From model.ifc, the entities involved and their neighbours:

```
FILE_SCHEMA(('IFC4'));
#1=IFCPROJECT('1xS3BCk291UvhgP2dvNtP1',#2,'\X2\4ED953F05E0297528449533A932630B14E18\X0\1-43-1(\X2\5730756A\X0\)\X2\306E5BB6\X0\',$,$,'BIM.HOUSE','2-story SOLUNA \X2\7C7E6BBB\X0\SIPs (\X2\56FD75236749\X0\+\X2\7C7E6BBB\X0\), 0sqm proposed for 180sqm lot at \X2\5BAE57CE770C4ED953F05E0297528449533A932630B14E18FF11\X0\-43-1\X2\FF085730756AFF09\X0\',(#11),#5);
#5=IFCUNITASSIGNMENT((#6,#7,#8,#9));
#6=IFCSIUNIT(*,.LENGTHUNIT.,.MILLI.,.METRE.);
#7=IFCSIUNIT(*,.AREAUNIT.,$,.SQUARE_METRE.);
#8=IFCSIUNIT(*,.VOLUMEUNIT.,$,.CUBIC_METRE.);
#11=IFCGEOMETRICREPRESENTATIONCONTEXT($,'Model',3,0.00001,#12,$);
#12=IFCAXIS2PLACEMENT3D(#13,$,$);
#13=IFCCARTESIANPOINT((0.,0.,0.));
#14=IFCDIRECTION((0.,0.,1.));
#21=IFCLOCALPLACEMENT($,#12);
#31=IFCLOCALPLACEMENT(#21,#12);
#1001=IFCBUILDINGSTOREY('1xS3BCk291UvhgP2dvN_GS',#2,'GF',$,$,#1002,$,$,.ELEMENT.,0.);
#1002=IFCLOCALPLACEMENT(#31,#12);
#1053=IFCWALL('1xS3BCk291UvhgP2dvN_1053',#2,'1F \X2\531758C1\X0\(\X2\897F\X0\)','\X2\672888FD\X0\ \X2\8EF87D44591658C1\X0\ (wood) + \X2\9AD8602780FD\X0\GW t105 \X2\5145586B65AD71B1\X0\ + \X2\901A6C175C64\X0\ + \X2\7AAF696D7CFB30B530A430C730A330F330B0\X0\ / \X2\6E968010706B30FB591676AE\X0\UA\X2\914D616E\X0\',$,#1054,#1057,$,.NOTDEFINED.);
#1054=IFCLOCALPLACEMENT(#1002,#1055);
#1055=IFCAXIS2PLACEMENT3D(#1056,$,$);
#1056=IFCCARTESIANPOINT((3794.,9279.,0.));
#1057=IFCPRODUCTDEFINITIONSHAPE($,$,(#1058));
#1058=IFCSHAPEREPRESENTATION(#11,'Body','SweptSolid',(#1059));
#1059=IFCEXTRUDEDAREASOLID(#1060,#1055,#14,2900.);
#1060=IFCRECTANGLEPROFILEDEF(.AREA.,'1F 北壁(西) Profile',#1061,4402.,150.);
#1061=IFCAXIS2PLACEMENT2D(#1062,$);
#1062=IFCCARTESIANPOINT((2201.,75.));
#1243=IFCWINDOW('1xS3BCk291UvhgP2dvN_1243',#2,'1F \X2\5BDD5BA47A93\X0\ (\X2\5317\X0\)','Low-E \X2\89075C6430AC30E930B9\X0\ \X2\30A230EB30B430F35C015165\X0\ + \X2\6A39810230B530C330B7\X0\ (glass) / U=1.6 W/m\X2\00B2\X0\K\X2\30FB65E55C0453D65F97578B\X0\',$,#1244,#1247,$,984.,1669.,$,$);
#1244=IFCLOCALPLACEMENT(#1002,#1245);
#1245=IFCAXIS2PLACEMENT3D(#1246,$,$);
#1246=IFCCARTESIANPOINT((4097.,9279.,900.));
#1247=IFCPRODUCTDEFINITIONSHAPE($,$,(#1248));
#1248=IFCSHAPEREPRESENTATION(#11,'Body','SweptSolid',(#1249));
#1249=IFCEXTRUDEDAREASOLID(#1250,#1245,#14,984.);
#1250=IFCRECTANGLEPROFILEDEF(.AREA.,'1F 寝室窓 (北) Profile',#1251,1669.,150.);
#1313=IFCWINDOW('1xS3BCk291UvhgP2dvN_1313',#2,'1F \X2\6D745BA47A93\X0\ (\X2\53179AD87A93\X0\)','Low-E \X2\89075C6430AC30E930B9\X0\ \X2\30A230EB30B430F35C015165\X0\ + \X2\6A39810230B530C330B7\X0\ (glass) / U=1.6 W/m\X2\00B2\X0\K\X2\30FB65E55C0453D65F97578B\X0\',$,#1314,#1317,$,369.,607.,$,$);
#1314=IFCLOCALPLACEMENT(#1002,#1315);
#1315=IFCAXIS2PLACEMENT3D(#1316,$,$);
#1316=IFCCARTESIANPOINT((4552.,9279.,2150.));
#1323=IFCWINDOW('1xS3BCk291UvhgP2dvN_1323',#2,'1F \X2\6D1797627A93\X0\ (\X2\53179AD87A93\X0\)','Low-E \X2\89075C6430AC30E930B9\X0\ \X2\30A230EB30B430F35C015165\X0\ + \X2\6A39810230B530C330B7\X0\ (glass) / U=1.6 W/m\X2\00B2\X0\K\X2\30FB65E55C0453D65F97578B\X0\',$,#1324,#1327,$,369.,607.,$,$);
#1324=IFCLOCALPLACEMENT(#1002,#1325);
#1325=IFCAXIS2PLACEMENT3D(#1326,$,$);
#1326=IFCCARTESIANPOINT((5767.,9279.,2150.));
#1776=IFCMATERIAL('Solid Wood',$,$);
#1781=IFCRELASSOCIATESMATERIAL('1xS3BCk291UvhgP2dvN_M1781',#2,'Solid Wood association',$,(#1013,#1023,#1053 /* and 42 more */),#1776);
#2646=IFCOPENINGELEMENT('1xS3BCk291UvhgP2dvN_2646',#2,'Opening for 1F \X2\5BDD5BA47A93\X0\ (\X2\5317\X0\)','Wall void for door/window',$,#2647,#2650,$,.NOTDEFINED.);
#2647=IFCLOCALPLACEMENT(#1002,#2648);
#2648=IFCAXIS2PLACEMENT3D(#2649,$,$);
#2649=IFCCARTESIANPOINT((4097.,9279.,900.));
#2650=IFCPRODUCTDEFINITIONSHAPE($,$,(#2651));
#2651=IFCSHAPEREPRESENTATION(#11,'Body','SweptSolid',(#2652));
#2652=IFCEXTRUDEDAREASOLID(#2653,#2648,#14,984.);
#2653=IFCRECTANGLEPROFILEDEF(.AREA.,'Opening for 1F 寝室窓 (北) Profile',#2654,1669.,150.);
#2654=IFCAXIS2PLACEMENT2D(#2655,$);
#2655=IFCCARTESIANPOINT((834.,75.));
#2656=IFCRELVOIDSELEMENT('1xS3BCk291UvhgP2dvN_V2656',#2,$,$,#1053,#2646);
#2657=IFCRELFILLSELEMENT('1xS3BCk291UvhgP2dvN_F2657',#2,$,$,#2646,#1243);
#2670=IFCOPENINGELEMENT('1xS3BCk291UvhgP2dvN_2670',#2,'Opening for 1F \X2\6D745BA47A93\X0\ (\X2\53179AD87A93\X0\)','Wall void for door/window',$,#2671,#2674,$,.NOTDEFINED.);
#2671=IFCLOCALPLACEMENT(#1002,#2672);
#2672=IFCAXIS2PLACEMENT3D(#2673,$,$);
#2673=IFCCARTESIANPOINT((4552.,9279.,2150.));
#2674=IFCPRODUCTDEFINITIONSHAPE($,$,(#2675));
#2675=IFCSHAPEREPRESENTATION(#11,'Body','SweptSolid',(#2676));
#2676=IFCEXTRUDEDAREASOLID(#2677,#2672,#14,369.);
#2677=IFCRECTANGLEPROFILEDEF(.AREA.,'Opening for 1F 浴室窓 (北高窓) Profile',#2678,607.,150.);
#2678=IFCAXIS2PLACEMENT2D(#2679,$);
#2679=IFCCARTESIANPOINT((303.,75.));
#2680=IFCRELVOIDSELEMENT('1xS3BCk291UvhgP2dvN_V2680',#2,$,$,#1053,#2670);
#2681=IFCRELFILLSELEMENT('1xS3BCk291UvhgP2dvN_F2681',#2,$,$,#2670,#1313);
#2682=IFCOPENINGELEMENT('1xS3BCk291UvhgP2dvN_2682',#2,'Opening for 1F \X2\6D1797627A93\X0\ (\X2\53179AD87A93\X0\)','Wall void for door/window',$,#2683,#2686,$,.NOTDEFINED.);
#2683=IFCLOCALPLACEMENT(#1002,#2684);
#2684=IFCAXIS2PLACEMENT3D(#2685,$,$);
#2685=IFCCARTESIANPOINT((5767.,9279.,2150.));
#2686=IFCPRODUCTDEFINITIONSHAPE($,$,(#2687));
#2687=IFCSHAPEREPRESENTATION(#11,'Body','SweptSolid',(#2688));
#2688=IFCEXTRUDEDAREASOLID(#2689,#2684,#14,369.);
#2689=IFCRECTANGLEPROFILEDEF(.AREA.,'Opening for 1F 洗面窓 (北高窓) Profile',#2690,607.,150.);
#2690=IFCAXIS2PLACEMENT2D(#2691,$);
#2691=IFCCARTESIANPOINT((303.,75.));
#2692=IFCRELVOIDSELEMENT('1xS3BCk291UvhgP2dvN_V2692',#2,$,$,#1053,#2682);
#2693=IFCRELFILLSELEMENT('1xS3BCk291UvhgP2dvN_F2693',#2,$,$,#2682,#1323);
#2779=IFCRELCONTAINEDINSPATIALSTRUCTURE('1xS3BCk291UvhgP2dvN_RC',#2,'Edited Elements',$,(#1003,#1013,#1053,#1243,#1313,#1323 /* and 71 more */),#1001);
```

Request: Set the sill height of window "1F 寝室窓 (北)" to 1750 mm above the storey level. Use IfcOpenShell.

```python
import numpy as np
import ifcopenshell
import ifcopenshell.api.geometry
import ifcopenshell.geom
import ifcopenshell.util.element
import ifcopenshell.util.placement
import ifcopenshell.util.shape
import ifcopenshell.util.unit

model = ifcopenshell.open("model.ifc")
unit_scale = ifcopenshell.util.unit.calculate_unit_scale(model)

window = model.by_id(1243)
opening = window.FillsVoids[0].RelatingOpeningElement
storey = ifcopenshell.util.element.get_container(window, ifc_class="IfcBuildingStorey")
level = ifcopenshell.util.placement.get_local_placement(storey.ObjectPlacement)[2, 3]

# The opening's origin need not be at the sill, so measure its lowest point.
shape = ifcopenshell.geom.create_shape(ifcopenshell.geom.settings(), opening)
bottom = ifcopenshell.util.shape.get_shape_bottom_elevation(shape, shape.geometry) / unit_scale
dz = level + 1.75 / unit_scale - bottom

shift = np.array([0.0, 0.0, dz])
# The window is not placed relative to its opening, so move both.
for product in (opening, window):
    matrix = ifcopenshell.util.placement.get_local_placement(product.ObjectPlacement)
    matrix[:3, 3] += shift
    ifcopenshell.api.geometry.edit_object_placement(model, product=product, matrix=matrix, is_si=False)

print(f"moved by {dz * unit_scale:+.3f} m")

model.write("model_rev.ifc")
```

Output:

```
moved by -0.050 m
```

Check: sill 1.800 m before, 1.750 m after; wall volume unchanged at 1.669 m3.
